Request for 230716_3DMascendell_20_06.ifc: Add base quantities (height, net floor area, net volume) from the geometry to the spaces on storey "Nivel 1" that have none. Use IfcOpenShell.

First a look at what the model holds.

```python
import ifcopenshell
import ifcopenshell.util.element
import ifcopenshell.util.unit

model = ifcopenshell.open("230716_3DMascendell_20_06.ifc")
print(model.schema)
for unit_type in ("LENGTHUNIT", "AREAUNIT", "VOLUMEUNIT"):
    print(unit_type, ifcopenshell.util.unit.calculate_unit_scale(model, unit_type))
storey = next(s for s in model.by_type("IfcBuildingStorey") if s.Name == "Nivel 1")
spaces = [e for e in ifcopenshell.util.element.get_decomposition(storey) if e.is_a("IfcSpace")]
for e in sorted(spaces, key=lambda e: e.id()):
    print(e.id(), e.is_a(), e.Name, list(ifcopenshell.util.element.get_psets(e, qtos_only=True)), sep=" | ")
```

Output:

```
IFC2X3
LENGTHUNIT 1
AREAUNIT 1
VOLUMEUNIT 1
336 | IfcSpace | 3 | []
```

```python
import ifcopenshell
import ifcopenshell.api.pset
import ifcopenshell.geom
import ifcopenshell.util.element
import ifcopenshell.util.shape
import ifcopenshell.util.unit

model = ifcopenshell.open("230716_3DMascendell_20_06.ifc")
unit_scale = ifcopenshell.util.unit.calculate_unit_scale(model)
area_scale = ifcopenshell.util.unit.calculate_unit_scale(model, "AREAUNIT")
volume_scale = ifcopenshell.util.unit.calculate_unit_scale(model, "VOLUMEUNIT")
settings = ifcopenshell.geom.settings()

storey = next(s for s in model.by_type("IfcBuildingStorey") if s.Name == "Nivel 1")
spaces = [e for e in ifcopenshell.util.element.get_decomposition(storey) if e.is_a("IfcSpace")]

for e in sorted(spaces, key=lambda e: e.id()):
    if ifcopenshell.util.element.get_psets(e, qtos_only=True, should_inherit=False):
        continue
    # Geometry comes back in metres, in the element's own axes.
    shape = ifcopenshell.geom.create_shape(settings, e)
    values = {
        "Height": ifcopenshell.util.shape.get_z(shape.geometry) / unit_scale,
        "NetFloorArea": ifcopenshell.util.shape.get_footprint_area(shape.geometry) / area_scale,
        "NetVolume": ifcopenshell.util.shape.get_volume(shape.geometry) / volume_scale,
    }
    qto = ifcopenshell.api.pset.add_qto(model, product=e, name="BaseQuantities")
    ifcopenshell.api.pset.edit_qto(model, qto=qto, properties=values)
    print(e.id(), {k: round(v, 3) for k, v in values.items()})

model.write("230716_3DMascendell_20_06_edited.ifc")
```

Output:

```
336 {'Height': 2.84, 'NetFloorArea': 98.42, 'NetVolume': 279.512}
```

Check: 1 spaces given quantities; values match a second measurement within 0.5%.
